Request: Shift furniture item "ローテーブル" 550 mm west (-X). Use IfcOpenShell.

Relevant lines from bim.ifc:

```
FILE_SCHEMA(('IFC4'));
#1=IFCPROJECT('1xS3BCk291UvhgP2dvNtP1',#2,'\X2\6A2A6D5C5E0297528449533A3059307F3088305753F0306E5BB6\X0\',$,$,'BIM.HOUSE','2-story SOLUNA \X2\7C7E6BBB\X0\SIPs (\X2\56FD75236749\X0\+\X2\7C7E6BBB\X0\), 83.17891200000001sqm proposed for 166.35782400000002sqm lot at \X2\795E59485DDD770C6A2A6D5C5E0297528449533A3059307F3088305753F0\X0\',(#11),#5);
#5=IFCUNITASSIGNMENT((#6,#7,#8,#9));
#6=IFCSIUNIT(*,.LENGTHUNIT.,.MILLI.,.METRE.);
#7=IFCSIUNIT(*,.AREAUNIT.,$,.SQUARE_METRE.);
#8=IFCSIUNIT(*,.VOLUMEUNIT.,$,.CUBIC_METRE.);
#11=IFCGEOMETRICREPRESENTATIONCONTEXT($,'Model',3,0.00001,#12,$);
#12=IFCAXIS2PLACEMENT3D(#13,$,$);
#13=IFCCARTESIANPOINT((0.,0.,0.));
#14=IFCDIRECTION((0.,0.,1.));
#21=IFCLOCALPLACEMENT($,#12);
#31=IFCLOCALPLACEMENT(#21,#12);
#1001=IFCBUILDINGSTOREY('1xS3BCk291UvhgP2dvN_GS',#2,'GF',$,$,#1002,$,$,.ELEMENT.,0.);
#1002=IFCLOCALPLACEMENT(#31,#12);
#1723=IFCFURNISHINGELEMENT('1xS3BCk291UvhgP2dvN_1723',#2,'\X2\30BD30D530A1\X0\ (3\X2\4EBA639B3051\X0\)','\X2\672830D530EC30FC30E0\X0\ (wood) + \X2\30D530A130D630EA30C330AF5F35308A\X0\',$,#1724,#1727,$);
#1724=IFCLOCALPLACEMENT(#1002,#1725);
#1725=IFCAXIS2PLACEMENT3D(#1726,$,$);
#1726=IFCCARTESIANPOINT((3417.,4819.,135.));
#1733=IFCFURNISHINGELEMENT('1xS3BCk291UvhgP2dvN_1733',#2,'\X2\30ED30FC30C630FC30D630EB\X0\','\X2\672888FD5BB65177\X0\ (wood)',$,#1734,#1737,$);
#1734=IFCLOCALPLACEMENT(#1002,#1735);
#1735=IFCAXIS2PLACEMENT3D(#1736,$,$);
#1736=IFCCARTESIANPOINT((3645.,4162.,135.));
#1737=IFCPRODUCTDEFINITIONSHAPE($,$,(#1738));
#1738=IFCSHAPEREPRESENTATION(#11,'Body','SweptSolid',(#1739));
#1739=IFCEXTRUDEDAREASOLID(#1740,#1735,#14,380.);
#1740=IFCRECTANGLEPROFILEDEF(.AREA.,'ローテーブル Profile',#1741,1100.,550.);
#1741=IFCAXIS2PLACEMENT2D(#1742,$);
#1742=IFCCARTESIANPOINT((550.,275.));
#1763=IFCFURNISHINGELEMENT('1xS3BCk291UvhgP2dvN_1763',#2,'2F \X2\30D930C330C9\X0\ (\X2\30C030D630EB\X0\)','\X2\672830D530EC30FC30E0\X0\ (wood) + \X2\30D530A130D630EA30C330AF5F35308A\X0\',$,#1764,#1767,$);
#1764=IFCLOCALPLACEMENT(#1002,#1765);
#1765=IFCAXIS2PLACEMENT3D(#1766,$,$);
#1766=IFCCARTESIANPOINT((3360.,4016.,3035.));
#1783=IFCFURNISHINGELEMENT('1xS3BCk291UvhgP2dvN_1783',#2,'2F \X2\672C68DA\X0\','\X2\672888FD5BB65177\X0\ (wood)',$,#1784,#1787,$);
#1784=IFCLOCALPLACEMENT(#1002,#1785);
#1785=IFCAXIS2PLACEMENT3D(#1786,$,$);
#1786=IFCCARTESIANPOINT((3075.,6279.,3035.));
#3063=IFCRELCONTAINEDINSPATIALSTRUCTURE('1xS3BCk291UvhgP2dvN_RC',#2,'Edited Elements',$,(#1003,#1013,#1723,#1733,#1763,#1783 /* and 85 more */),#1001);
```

```python
import ifcopenshell
import ifcopenshell.api.geometry
import ifcopenshell.util.placement

model = ifcopenshell.open("bim.ifc")

item = model.by_guid("1xS3BCk291UvhgP2dvN_1733")
matrix = ifcopenshell.util.placement.get_local_placement(item.ObjectPlacement)
matrix[0, 3] -= 550.0
ifcopenshell.api.geometry.edit_object_placement(model, product=item, matrix=matrix, is_si=False)

print(ifcopenshell.util.placement.get_local_placement(item.ObjectPlacement).round(3) + 0.0)

model.write("bim_v2.ifc")
```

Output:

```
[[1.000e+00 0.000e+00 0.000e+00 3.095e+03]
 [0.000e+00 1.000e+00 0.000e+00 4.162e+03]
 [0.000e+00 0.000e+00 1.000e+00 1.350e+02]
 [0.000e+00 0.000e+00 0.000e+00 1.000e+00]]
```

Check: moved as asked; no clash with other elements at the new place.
